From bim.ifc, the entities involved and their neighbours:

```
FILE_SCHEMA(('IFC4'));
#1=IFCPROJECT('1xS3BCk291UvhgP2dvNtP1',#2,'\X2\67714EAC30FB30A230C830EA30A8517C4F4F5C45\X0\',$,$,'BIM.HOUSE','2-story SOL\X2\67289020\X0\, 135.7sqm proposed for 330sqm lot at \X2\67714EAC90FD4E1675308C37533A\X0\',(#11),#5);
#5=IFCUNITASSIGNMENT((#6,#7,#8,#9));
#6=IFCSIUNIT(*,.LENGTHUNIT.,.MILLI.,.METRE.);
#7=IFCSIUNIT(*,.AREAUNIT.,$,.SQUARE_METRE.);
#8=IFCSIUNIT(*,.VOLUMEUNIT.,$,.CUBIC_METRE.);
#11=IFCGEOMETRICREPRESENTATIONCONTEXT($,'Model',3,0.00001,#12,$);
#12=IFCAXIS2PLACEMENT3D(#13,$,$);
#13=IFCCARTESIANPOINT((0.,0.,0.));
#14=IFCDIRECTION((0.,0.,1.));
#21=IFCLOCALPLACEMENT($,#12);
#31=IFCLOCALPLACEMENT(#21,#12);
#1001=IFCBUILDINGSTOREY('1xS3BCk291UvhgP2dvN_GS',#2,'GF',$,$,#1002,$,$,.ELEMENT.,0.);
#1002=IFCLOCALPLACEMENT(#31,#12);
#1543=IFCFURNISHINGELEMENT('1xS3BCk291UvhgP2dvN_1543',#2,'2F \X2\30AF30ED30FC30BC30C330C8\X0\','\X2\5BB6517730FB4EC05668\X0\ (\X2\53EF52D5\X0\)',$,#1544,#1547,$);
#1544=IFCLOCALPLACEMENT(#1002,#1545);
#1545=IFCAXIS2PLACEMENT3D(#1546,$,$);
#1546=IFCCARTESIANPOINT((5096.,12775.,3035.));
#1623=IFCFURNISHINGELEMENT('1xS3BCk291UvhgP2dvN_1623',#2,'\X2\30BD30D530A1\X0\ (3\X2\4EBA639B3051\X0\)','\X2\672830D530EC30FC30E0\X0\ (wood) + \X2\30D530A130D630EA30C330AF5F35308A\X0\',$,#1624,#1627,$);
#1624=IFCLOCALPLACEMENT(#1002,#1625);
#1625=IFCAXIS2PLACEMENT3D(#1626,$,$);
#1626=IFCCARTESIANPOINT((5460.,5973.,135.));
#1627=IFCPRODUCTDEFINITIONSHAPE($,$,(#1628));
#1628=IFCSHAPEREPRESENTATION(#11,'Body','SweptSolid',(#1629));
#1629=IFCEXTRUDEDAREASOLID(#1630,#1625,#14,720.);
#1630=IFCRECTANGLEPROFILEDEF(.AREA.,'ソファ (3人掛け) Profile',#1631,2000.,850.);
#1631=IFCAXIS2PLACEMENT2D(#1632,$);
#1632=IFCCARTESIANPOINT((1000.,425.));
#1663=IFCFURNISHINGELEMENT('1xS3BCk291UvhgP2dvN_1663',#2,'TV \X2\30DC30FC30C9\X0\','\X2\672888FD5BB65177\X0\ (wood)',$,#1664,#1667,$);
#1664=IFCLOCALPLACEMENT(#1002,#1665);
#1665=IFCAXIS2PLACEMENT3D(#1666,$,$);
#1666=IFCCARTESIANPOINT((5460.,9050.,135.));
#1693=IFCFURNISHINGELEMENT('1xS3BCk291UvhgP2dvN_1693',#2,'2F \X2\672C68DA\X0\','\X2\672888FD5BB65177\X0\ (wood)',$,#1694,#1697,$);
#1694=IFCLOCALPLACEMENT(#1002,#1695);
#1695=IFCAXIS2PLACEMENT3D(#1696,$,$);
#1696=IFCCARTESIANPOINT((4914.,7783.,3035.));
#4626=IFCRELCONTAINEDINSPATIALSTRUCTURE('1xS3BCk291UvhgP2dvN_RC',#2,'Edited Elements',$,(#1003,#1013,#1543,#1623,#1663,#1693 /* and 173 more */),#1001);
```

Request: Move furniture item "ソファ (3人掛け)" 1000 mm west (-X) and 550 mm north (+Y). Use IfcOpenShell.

```python
import ifcopenshell
import ifcopenshell.api.geometry
import ifcopenshell.util.placement

model = ifcopenshell.open("bim.ifc")

item = model.by_id(1623)
matrix = ifcopenshell.util.placement.get_local_placement(item.ObjectPlacement)
matrix[0, 3] -= 1000.0
matrix[1, 3] += 550.0
ifcopenshell.api.geometry.edit_object_placement(model, product=item, matrix=matrix, is_si=False)

print(ifcopenshell.util.placement.get_local_placement(item.ObjectPlacement).round(3) + 0.0)

model.write("bim_rev.ifc")
```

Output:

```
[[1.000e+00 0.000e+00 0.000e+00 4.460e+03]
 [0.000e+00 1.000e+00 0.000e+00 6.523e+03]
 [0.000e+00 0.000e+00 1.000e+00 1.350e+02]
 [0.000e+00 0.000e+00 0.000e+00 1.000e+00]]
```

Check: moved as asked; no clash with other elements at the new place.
